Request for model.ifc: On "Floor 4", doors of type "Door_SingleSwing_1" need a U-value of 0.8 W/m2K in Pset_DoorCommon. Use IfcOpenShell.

First a look at what the model holds.

```python
import ifcopenshell
import ifcopenshell.util.element

model = ifcopenshell.open("model.ifc")
print(model.schema)
storey = next(s for s in model.by_type("IfcBuildingStorey") if s.Name == "Floor 4")
doors = [e for e in ifcopenshell.util.element.get_decomposition(storey) if e.is_a("IfcDoor")]
seen = {}
for e in doors:
    element_type = ifcopenshell.util.element.get_type(e)
    key = (element_type.Name if element_type != e and element_type else None, ifcopenshell.util.element.get_pset(e, "Pset_DoorCommon", "ThermalTransmittance"))
    seen[key] = seen.get(key, 0) + 1
for (name, value), count in sorted(seen.items(), key=str):
    print(count, "x", name, "|", value)
```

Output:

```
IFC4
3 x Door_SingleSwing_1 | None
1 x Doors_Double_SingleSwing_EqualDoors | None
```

```python
import ifcopenshell
import ifcopenshell.api.pset
import ifcopenshell.util.element

model = ifcopenshell.open("model.ifc")

storey = next(s for s in model.by_type("IfcBuildingStorey") if s.Name == "Floor 4")
doors = [e for e in ifcopenshell.util.element.get_decomposition(storey) if e.is_a("IfcDoor")]

count = 0
for e in doors:
    element_type = ifcopenshell.util.element.get_type(e)
    if element_type in (None, e) or element_type.Name != "Door_SingleSwing_1":
        continue
    # add_pset returns the element's existing set when there is one.
    pset = ifcopenshell.api.pset.add_pset(model, product=e, name="Pset_DoorCommon")
    ifcopenshell.api.pset.edit_pset(model, pset=pset, properties={"ThermalTransmittance": 0.8})
    count += 1

print(count, "doors updated")

model.write("model_updated.ifc")
```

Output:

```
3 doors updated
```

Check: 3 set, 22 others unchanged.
